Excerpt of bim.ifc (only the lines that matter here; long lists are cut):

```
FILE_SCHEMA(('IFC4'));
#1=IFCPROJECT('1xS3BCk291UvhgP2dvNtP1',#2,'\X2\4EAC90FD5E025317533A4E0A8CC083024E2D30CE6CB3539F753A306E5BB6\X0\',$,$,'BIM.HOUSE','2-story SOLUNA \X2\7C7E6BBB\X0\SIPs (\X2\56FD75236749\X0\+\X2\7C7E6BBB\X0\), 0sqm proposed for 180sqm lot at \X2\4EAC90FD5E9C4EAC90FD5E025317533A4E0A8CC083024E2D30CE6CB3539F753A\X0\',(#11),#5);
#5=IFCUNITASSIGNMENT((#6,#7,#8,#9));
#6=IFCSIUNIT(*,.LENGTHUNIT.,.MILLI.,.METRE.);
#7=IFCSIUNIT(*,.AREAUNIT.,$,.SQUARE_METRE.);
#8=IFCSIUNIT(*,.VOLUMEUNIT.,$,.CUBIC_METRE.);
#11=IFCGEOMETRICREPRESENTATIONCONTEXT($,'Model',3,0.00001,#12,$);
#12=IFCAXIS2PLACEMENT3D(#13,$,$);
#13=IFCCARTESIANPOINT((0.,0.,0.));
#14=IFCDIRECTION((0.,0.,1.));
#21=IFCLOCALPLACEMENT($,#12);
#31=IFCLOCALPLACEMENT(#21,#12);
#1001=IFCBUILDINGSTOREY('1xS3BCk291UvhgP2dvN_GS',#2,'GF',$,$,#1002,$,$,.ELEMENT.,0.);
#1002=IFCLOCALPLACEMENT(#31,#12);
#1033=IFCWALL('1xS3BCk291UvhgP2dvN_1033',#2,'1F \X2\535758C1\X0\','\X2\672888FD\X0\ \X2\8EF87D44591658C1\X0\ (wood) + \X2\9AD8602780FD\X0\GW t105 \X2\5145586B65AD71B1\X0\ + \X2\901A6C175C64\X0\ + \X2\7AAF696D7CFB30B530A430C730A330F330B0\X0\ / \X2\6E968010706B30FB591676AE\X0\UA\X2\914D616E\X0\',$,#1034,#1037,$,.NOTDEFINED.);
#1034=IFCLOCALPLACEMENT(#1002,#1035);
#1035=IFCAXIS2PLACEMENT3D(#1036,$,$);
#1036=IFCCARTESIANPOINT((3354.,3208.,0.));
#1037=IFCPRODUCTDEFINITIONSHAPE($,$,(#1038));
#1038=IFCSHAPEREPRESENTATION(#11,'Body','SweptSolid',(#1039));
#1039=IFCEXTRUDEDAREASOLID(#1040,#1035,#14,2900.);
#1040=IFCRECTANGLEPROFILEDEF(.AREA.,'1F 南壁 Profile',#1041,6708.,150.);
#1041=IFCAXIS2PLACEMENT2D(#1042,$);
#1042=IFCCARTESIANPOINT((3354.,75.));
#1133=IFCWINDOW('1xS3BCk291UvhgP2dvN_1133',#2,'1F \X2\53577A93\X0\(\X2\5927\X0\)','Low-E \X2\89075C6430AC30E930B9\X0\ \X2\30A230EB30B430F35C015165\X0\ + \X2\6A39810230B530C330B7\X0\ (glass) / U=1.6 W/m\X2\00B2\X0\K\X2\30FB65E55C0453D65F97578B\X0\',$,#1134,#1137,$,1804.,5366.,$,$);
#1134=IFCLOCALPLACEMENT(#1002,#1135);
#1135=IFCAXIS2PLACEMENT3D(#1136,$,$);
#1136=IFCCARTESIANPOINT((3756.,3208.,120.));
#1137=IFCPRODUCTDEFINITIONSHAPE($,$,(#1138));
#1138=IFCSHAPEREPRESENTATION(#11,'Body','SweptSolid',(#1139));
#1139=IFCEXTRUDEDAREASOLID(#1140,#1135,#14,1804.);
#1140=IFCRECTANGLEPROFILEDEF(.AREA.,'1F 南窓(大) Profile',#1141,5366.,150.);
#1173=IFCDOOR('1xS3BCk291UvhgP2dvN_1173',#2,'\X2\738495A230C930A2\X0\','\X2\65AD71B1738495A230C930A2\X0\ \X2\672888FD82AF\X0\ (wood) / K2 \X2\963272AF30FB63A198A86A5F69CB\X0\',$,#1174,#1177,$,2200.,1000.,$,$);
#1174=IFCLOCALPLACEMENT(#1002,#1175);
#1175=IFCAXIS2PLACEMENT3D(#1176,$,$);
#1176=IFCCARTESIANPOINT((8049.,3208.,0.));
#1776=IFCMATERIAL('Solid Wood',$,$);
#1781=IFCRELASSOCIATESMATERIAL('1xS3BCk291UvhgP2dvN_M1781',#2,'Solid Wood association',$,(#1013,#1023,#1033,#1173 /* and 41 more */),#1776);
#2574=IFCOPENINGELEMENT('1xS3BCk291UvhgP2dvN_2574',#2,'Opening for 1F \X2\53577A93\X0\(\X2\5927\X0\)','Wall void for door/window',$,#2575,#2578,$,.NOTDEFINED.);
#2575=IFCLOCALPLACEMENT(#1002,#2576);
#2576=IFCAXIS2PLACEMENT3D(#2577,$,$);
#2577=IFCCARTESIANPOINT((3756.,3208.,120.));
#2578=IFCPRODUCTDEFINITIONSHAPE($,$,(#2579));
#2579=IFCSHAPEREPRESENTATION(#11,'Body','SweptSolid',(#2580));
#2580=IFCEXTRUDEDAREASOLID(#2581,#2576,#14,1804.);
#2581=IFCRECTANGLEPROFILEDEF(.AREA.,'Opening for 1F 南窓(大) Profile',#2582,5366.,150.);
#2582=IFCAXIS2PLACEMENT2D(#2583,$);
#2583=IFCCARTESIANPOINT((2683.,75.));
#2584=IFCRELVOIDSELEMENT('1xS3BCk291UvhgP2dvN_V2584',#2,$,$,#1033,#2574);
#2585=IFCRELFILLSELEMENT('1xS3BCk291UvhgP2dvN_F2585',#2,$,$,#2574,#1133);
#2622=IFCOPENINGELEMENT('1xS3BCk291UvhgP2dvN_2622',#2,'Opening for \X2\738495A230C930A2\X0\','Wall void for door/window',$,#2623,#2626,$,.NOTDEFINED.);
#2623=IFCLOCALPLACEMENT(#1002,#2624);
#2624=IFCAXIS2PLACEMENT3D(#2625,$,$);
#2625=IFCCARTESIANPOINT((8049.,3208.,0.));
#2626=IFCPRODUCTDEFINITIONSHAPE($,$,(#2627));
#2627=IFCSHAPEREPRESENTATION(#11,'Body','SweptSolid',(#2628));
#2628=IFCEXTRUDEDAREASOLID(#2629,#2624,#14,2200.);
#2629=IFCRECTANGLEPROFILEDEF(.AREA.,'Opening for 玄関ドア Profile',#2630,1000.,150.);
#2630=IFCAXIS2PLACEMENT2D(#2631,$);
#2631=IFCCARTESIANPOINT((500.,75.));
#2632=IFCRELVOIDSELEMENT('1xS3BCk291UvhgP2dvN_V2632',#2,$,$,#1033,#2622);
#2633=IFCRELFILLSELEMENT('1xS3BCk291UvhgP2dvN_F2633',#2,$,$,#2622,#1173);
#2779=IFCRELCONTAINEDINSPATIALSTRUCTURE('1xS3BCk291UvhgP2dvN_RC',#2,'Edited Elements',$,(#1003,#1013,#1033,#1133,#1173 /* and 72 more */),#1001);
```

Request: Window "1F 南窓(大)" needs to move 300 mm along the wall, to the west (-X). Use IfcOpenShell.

```python
import ifcopenshell
import ifcopenshell.api.geometry
import ifcopenshell.util.placement
import ifcopenshell.util.unit

model = ifcopenshell.open("bim.ifc")
unit_scale = ifcopenshell.util.unit.calculate_unit_scale(model)

window = model.by_guid("1xS3BCk291UvhgP2dvN_1133")
opening = window.FillsVoids[0].RelatingOpeningElement
wall = opening.VoidsElements[0].RelatingBuildingElement

wall_matrix = ifcopenshell.util.placement.get_local_placement(wall.ObjectPlacement)
shift = wall_matrix[:3, 0] * -0.3 / unit_scale
before = ifcopenshell.util.placement.get_local_placement(window.ObjectPlacement)[:3, 3].copy()

# The window is not placed relative to its opening, so move both.
for product in (opening, window):
    matrix = ifcopenshell.util.placement.get_local_placement(product.ObjectPlacement)
    matrix[:3, 3] += shift
    ifcopenshell.api.geometry.edit_object_placement(model, product=product, matrix=matrix, is_si=False)

after = ifcopenshell.util.placement.get_local_placement(window.ObjectPlacement)[:3, 3]
print("window moved by", (after - before).round(3) + 0.0)

model.write("bim_rev.ifc")
```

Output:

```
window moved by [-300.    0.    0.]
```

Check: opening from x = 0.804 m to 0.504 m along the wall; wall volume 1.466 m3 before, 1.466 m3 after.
